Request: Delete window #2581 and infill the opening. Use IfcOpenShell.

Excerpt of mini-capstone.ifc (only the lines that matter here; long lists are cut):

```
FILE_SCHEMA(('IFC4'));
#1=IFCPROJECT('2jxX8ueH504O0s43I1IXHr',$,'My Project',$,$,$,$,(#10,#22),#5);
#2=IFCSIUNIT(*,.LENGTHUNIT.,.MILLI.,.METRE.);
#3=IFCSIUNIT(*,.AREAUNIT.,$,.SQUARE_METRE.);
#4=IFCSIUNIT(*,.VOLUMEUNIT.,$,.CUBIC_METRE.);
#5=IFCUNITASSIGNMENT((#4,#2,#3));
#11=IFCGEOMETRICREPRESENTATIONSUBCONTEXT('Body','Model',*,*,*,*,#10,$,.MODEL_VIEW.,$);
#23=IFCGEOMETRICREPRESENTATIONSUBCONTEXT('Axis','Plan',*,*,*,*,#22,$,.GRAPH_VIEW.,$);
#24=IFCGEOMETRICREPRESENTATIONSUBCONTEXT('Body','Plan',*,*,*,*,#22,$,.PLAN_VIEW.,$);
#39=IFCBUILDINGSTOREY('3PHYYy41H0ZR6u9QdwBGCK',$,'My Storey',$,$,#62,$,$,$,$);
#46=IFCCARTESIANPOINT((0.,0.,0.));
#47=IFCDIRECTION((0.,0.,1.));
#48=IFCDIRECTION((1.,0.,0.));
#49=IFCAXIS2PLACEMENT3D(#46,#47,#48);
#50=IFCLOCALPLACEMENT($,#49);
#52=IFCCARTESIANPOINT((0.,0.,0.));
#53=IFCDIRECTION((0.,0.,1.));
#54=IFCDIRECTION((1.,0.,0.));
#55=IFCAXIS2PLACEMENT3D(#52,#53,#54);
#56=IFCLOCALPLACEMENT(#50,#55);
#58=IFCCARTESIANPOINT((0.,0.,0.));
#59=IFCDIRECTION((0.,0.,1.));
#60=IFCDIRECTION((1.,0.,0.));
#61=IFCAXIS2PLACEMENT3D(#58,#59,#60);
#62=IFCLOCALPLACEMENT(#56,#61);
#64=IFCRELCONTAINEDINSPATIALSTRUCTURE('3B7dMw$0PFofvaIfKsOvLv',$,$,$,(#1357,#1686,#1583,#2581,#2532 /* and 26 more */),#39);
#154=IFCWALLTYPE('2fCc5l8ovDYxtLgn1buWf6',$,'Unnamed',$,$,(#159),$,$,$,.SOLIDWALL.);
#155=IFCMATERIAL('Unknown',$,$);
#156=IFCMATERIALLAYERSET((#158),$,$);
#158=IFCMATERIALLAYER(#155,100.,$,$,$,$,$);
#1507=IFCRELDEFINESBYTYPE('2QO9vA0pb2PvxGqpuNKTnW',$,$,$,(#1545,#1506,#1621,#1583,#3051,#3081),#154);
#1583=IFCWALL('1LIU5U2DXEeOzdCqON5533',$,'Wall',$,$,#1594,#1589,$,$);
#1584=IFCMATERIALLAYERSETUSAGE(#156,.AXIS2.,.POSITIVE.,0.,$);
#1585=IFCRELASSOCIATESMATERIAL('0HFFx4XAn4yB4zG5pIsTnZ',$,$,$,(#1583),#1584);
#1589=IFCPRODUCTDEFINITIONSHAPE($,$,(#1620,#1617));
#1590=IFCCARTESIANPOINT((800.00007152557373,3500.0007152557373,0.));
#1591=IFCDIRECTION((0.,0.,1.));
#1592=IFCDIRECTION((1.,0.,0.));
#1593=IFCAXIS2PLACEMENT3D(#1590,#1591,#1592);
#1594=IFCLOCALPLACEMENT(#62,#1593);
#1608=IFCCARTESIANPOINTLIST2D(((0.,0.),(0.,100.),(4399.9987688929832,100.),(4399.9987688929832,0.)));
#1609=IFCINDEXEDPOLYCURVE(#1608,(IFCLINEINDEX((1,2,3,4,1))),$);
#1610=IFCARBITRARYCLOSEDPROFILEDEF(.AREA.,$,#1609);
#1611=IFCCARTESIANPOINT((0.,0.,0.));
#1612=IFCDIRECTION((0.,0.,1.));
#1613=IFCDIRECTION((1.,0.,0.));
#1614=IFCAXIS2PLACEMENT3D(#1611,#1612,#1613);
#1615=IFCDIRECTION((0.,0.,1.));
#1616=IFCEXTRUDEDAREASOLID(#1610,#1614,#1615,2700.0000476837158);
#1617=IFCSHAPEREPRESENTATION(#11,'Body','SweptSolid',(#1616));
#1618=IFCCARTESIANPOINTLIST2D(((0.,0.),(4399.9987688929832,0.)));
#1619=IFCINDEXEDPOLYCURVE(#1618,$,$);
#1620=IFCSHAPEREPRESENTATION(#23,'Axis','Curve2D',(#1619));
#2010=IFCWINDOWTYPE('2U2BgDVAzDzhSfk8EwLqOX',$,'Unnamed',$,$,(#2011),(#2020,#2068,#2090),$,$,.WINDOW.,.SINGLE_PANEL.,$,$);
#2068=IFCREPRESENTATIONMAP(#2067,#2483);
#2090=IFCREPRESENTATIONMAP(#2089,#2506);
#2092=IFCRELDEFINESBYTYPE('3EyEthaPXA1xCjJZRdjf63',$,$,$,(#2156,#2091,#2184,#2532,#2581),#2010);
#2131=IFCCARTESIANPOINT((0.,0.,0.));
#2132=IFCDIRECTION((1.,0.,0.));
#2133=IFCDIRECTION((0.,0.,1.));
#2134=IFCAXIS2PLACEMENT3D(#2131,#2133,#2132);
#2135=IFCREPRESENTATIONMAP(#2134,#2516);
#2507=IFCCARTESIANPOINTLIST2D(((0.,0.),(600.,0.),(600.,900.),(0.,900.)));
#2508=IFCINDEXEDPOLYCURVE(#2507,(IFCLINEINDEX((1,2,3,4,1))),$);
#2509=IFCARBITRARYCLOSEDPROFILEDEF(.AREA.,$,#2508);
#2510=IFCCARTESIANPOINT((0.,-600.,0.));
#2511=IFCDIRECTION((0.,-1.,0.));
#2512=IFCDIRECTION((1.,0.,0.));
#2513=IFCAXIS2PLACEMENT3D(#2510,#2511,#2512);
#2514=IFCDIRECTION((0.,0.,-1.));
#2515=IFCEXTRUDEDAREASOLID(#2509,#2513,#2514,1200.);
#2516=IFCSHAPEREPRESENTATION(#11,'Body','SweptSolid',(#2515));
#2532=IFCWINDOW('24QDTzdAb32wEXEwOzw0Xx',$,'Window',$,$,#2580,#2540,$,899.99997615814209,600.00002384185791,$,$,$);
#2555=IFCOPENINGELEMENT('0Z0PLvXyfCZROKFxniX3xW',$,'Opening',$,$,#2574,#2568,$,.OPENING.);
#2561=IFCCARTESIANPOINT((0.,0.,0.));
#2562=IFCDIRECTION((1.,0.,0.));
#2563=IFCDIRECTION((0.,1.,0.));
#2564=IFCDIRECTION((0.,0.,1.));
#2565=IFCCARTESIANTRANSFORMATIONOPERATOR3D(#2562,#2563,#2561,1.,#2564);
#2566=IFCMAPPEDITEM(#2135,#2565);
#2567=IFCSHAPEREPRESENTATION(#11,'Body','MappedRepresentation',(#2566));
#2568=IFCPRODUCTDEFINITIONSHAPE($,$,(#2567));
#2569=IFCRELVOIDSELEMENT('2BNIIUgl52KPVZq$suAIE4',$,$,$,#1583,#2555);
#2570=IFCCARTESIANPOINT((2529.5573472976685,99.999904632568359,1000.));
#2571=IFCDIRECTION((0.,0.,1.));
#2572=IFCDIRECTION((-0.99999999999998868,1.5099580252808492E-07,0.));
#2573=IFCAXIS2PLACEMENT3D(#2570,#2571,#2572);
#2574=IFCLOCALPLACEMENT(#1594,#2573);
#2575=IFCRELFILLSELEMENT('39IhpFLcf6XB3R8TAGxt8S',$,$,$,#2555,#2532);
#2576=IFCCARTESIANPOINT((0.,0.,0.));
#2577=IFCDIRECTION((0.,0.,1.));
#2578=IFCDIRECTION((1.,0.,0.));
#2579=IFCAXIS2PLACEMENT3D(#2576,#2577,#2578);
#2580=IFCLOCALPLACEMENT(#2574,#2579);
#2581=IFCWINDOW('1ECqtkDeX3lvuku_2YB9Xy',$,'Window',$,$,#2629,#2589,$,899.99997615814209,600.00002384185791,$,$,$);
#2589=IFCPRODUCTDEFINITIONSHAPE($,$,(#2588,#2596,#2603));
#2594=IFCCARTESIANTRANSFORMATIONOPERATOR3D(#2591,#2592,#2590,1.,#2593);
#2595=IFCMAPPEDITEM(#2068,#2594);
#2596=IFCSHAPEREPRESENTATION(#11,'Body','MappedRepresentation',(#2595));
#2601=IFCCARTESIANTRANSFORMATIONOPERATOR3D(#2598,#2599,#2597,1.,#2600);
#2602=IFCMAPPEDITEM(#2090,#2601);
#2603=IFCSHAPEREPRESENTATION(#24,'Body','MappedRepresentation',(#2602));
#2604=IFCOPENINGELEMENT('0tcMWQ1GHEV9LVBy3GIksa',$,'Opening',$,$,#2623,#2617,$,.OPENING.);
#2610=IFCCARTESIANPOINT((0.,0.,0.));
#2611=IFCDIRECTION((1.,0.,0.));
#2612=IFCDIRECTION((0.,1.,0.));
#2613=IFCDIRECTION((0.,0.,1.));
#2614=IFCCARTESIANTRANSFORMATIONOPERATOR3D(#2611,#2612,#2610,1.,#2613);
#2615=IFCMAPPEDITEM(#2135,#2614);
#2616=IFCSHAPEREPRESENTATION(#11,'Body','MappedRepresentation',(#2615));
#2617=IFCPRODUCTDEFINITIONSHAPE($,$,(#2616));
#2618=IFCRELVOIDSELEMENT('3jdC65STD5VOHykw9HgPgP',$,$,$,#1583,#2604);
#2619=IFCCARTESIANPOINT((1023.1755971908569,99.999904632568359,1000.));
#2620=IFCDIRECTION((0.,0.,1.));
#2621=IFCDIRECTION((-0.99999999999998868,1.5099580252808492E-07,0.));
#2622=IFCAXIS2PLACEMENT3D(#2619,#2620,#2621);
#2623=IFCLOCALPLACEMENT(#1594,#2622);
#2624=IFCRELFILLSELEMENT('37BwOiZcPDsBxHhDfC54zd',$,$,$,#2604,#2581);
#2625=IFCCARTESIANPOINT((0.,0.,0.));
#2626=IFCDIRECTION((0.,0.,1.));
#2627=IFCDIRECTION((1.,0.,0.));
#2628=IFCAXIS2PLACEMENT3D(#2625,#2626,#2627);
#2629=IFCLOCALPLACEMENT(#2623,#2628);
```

```python
import ifcopenshell
import ifcopenshell.api.feature
import ifcopenshell.api.root
import ifcopenshell.geom
import ifcopenshell.util.shape

model = ifcopenshell.open("mini-capstone.ifc")
settings = ifcopenshell.geom.settings()


def volume(element):
    """Net volume in cubic metres, openings subtracted."""
    shape = ifcopenshell.geom.create_shape(settings, element)
    return ifcopenshell.util.shape.get_volume(shape.geometry)


window = model.by_guid("1ECqtkDeX3lvuku_2YB9Xy")
opening = window.FillsVoids[0].RelatingOpeningElement
wall = opening.VoidsElements[0].RelatingBuildingElement
before = volume(wall)

ifcopenshell.api.root.remove_product(model, product=window)
ifcopenshell.api.feature.remove_feature(model, feature=opening)

after = volume(wall)

print(f"wall volume {before:.3f} -> {after:.3f} m3")

model.write("mini-capstone_rev.ifc")
```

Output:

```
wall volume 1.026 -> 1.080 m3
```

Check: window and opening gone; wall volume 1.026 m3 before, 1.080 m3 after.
